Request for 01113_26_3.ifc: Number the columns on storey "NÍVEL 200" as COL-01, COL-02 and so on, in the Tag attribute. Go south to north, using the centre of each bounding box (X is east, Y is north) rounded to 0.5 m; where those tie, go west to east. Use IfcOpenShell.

First a look at what the model holds.

```python
import ifcopenshell
import ifcopenshell.util.element
import ifcopenshell.util.placement

model = ifcopenshell.open("01113_26_3.ifc")
print(model.schema)
storey = next(s for s in model.by_type("IfcBuildingStorey") if s.Name == "NÍVEL 200")
columns = [e for e in ifcopenshell.util.element.get_decomposition(storey) if e.is_a("IfcColumn")]
for e in sorted(columns, key=lambda e: e.id()):
    origin = ifcopenshell.util.placement.get_local_placement(e.ObjectPlacement)[:3, 3]
    print(e.id(), e.Tag, e.Name, origin.round(2) + 0.0, sep=" | ")
```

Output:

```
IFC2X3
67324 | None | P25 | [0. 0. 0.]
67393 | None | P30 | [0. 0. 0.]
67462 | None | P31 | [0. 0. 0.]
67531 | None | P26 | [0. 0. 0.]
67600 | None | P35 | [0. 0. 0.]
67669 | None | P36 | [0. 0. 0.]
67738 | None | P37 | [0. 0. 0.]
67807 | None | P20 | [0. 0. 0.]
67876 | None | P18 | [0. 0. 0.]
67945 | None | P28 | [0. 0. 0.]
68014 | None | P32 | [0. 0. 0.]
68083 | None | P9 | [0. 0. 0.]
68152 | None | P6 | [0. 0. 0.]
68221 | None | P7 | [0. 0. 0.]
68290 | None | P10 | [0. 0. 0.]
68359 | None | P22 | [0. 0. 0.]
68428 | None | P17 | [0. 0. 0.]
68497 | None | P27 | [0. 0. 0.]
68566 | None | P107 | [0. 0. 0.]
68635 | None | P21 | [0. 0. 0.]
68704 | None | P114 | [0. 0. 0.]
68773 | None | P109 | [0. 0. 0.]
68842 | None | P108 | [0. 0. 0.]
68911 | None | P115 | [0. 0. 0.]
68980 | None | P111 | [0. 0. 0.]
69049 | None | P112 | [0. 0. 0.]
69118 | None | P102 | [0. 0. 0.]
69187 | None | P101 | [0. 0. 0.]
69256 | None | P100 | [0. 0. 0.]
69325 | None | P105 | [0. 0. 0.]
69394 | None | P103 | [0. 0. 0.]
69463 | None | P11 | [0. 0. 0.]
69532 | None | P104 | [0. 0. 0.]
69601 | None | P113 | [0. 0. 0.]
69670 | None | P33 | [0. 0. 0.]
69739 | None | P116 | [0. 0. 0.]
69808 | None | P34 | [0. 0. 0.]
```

```python
import ifcopenshell
import ifcopenshell.geom
import ifcopenshell.util.element
import ifcopenshell.util.shape

model = ifcopenshell.open("01113_26_3.ifc")
settings = ifcopenshell.geom.settings()
settings.set("use-world-coords", True)


def centre(element):
    shape = ifcopenshell.geom.create_shape(settings, element)
    return ifcopenshell.util.shape.get_bbox_centroid(shape.geometry)


storey = next(s for s in model.by_type("IfcBuildingStorey") if s.Name == "NÍVEL 200")
columns = [e for e in ifcopenshell.util.element.get_decomposition(storey) if e.is_a("IfcColumn")]

# Insertion points can sit at a corner or the storey origin, so sort by the geometry (in metres).
centres = {e: centre(e) for e in columns}
columns.sort(key=lambda e: (round(centres[e][1] / 0.5), centres[e][0]))

for i, e in enumerate(columns, start=1):
    number = f"COL-{i:02d}"
    e.Tag = number
    print(e.id(), number)

model.write("01113_26_3_rev.ifc")
```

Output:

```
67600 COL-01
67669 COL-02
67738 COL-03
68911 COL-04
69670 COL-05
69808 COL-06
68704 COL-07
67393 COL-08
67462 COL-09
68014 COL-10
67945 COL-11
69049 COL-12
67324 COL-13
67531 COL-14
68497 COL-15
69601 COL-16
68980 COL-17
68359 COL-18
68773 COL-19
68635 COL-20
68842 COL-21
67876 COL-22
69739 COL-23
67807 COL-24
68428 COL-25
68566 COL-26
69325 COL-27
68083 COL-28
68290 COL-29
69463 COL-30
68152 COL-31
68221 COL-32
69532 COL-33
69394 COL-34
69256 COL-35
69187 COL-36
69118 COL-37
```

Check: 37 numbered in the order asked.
